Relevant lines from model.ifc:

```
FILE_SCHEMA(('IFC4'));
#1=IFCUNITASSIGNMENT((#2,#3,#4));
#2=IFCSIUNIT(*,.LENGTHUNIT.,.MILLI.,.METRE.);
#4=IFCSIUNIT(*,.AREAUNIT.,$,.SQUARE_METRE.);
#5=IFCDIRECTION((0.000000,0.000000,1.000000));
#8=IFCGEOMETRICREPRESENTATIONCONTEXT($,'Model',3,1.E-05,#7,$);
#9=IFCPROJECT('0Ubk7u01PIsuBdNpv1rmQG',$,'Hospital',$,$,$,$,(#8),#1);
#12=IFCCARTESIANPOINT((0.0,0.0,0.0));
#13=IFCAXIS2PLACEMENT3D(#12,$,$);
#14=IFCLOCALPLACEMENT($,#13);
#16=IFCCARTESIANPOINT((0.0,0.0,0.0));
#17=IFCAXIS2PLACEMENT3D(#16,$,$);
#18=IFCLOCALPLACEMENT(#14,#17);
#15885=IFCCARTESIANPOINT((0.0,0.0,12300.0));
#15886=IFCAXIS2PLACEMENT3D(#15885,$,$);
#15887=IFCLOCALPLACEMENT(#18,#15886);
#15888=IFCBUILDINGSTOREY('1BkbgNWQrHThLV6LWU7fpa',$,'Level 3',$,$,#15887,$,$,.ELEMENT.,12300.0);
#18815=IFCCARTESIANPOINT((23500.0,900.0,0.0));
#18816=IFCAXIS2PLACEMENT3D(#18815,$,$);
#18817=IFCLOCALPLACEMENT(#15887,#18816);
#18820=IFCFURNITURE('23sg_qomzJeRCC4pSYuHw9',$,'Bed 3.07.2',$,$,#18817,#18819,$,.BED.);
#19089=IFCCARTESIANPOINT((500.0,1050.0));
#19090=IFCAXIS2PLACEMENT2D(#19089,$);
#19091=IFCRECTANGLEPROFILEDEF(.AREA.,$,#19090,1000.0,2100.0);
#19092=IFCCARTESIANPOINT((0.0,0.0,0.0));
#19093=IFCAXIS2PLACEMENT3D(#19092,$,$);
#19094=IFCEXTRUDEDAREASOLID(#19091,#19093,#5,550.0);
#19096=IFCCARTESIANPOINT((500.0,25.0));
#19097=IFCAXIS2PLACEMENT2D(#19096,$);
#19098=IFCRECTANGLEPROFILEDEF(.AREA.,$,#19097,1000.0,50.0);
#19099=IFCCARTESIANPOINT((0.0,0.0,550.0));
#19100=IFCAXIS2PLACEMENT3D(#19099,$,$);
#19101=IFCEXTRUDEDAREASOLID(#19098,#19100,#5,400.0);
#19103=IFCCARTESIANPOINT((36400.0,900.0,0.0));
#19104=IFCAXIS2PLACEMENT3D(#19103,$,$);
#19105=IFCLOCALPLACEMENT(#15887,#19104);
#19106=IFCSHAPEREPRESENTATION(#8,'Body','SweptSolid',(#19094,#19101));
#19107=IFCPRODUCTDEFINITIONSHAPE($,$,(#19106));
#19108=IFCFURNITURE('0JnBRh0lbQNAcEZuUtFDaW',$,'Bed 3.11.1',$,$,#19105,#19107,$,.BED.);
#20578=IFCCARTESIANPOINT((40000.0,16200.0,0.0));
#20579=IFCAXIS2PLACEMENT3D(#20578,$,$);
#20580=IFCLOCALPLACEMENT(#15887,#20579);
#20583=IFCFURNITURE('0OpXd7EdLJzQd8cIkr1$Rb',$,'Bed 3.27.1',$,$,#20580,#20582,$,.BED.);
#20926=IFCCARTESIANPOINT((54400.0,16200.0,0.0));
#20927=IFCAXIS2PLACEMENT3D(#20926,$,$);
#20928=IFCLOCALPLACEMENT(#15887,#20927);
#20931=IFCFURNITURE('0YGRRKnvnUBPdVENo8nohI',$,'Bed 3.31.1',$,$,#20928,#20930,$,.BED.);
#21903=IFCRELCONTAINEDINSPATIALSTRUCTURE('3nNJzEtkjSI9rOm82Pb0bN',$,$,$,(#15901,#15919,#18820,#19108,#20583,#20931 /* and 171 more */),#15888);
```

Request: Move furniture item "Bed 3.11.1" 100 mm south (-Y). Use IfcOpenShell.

```python
import ifcopenshell
import ifcopenshell.api.geometry
import ifcopenshell.util.placement
import ifcopenshell.util.unit

model = ifcopenshell.open("model.ifc")
unit_scale = ifcopenshell.util.unit.calculate_unit_scale(model)

item = model.by_id(19108)
matrix = ifcopenshell.util.placement.get_local_placement(item.ObjectPlacement)
matrix[1, 3] -= 0.1 / unit_scale
ifcopenshell.api.geometry.edit_object_placement(model, product=item, matrix=matrix, is_si=False)

print(ifcopenshell.util.placement.get_local_placement(item.ObjectPlacement).round(3) + 0.0)

model.write("model_edited.ifc")
```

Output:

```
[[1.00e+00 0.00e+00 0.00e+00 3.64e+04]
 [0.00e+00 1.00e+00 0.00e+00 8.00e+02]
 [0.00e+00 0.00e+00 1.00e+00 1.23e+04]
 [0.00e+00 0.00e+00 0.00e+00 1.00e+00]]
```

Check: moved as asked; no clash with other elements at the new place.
